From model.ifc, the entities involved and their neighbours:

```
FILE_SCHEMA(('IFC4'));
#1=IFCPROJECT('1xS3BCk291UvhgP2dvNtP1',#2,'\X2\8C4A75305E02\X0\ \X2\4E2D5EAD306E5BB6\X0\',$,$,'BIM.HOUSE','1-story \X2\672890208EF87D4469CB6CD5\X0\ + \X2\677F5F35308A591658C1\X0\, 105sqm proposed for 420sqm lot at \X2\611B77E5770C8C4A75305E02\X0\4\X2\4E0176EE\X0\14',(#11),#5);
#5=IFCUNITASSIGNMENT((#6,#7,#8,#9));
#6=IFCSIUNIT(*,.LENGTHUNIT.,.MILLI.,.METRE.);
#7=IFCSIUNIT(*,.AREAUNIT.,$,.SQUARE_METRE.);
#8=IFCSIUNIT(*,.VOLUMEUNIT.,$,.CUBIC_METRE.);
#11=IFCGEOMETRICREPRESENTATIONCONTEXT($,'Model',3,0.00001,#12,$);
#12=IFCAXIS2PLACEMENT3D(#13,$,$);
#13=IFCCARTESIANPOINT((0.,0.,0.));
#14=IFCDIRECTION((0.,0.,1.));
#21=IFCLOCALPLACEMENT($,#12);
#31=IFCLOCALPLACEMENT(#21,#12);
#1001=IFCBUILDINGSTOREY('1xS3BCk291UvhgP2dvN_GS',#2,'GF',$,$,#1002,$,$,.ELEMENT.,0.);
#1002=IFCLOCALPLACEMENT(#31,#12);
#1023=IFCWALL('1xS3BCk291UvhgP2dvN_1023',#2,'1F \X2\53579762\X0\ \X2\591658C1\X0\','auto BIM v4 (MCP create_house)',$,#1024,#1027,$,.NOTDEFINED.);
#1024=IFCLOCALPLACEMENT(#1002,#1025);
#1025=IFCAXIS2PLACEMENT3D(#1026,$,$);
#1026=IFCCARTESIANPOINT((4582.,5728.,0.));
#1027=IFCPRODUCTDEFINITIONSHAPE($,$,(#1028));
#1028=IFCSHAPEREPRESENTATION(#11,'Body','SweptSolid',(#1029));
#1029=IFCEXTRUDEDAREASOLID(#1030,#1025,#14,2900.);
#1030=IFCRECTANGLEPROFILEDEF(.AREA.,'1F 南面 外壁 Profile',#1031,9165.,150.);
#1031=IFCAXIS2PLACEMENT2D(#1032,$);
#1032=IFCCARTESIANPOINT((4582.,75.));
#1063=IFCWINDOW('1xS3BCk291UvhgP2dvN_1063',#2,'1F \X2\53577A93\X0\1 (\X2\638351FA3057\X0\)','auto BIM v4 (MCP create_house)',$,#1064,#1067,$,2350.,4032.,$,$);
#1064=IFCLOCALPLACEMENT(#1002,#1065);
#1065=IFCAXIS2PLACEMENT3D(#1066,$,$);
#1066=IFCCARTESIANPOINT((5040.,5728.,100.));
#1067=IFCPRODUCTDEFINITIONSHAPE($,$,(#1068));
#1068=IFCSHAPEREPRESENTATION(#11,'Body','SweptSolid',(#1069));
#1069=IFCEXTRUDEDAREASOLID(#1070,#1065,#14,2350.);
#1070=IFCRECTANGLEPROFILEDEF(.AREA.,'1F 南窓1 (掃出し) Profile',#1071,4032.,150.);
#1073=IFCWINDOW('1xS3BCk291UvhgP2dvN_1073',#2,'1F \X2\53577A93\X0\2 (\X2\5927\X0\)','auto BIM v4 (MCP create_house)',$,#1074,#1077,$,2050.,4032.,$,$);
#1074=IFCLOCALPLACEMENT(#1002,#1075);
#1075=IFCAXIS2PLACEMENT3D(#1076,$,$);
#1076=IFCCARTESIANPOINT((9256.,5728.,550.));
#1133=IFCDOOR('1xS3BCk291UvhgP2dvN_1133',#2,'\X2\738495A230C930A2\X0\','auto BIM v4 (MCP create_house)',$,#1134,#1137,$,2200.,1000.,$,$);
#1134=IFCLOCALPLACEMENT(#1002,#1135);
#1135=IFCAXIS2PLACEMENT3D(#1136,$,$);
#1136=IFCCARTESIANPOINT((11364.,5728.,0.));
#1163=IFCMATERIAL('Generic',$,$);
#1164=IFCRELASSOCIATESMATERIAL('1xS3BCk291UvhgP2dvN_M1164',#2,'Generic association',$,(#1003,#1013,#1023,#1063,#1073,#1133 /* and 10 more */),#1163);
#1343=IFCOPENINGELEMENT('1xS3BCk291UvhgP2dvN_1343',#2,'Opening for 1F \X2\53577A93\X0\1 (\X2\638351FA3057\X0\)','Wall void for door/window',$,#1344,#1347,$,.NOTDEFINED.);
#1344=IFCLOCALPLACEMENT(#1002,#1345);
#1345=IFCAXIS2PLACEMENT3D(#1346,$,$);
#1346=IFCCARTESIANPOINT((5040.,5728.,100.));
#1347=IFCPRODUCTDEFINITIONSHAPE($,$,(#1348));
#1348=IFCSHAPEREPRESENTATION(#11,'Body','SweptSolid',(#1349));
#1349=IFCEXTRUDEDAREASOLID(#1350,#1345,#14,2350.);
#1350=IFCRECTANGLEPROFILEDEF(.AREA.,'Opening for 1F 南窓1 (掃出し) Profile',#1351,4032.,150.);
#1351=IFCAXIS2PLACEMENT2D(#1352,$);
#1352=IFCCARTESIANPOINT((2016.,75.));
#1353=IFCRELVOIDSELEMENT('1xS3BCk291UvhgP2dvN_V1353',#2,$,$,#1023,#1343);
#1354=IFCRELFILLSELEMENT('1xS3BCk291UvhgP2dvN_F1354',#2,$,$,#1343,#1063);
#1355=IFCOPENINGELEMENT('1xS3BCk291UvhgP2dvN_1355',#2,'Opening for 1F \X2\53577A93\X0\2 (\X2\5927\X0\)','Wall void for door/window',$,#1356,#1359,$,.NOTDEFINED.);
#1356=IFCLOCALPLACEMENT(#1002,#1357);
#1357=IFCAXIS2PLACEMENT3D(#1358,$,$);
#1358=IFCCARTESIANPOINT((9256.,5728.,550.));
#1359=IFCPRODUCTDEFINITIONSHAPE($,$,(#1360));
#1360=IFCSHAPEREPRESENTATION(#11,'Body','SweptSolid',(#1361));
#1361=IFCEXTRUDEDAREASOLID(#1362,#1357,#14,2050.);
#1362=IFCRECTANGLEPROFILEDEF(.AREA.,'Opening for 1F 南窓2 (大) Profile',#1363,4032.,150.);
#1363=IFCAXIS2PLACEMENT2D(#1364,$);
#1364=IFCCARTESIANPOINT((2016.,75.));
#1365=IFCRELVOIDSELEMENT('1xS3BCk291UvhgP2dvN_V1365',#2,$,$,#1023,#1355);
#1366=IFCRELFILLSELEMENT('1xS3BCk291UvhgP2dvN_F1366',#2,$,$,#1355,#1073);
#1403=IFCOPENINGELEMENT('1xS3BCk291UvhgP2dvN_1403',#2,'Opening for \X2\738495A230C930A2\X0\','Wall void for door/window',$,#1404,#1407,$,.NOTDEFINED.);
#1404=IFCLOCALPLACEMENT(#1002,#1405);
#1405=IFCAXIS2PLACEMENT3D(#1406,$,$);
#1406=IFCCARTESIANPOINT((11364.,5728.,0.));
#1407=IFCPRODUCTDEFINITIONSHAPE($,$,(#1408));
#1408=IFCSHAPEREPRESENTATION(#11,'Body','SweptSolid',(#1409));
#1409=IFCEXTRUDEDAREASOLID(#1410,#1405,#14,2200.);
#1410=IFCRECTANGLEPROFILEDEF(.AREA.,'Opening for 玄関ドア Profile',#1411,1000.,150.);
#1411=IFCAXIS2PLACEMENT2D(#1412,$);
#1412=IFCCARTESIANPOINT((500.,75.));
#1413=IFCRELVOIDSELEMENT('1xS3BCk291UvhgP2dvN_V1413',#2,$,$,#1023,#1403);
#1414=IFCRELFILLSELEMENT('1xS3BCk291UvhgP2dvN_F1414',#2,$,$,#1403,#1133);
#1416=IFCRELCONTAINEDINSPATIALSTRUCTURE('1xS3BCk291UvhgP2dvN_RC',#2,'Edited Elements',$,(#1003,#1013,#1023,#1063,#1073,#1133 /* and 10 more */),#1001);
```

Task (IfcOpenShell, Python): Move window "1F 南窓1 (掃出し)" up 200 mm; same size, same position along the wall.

```python
import numpy as np
import ifcopenshell
import ifcopenshell.api.geometry
import ifcopenshell.util.placement
import ifcopenshell.util.unit

model = ifcopenshell.open("model.ifc")
unit_scale = ifcopenshell.util.unit.calculate_unit_scale(model)

window = model.by_id(1063)
opening = window.FillsVoids[0].RelatingOpeningElement
dz = 200.0

shift = np.array([0.0, 0.0, dz])
# The window is not placed relative to its opening, so move both.
for product in (opening, window):
    matrix = ifcopenshell.util.placement.get_local_placement(product.ObjectPlacement)
    matrix[:3, 3] += shift
    ifcopenshell.api.geometry.edit_object_placement(model, product=product, matrix=matrix, is_si=False)

print(f"moved by {dz * unit_scale:+.3f} m")

model.write("model_edited.ifc")
```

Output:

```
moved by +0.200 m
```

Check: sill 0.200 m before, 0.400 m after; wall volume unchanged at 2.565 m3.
